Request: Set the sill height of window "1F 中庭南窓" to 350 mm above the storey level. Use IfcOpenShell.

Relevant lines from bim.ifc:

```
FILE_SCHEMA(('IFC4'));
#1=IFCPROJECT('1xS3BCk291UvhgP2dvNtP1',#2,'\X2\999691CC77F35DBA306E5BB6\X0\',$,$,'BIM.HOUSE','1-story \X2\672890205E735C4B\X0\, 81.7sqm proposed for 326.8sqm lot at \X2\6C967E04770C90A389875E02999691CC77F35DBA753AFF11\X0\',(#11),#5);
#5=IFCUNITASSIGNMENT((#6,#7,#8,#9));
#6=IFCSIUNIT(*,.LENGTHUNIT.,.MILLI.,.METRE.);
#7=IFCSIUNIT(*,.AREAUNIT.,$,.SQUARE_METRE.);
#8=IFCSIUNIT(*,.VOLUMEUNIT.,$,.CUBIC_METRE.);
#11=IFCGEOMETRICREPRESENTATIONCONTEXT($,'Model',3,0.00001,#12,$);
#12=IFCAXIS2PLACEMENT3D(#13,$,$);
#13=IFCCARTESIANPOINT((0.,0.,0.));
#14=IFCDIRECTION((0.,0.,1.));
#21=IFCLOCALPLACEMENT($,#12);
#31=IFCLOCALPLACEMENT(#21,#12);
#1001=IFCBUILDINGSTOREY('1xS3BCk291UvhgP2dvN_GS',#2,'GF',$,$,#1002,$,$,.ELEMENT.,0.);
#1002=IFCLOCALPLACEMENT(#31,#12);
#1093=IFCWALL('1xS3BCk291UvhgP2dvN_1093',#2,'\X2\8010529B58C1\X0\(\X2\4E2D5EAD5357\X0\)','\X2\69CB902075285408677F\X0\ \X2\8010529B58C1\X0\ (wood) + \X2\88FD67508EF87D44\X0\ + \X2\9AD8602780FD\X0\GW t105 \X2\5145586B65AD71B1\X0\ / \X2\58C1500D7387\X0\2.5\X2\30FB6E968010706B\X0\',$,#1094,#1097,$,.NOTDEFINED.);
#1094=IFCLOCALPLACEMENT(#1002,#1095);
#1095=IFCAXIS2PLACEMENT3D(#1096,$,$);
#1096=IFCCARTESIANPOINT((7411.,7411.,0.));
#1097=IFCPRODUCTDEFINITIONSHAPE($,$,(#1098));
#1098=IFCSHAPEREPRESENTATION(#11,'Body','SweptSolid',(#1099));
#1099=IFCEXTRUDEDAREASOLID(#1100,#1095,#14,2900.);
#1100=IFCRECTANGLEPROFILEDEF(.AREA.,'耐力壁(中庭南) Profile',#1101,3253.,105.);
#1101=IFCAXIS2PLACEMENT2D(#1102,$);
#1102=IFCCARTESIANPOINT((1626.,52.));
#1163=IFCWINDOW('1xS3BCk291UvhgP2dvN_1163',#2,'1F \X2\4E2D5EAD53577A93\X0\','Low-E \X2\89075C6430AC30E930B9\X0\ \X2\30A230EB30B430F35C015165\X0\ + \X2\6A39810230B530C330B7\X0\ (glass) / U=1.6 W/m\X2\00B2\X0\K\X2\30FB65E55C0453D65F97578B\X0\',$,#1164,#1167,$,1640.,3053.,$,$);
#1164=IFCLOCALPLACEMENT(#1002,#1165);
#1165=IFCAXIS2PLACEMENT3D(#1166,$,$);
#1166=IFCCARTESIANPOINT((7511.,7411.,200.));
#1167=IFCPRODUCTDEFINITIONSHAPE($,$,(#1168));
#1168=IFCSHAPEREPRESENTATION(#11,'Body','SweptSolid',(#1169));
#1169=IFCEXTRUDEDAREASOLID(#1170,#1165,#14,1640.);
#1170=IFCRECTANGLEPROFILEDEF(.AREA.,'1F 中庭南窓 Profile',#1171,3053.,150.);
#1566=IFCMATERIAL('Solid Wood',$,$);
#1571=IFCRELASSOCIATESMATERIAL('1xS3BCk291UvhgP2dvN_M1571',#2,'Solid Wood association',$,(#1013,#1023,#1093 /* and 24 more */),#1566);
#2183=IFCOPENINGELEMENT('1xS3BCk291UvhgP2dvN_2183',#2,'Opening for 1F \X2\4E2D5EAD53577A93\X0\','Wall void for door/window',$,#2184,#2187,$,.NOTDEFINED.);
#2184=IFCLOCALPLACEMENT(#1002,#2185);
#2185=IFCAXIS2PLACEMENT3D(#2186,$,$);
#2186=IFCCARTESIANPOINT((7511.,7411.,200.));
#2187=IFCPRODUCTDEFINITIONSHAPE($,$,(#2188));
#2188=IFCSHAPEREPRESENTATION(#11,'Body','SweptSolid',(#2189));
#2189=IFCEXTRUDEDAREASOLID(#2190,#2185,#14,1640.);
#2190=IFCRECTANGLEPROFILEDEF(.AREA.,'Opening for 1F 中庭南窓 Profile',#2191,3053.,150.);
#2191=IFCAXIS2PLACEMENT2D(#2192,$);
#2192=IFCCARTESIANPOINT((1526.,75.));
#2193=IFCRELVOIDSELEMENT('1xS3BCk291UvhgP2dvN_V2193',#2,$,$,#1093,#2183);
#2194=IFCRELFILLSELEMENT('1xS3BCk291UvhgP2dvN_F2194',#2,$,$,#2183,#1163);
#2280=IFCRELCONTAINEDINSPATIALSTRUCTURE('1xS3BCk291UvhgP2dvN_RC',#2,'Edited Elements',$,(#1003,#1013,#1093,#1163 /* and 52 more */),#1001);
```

```python
import numpy as np
import ifcopenshell
import ifcopenshell.api.geometry
import ifcopenshell.geom
import ifcopenshell.util.element
import ifcopenshell.util.placement
import ifcopenshell.util.shape
import ifcopenshell.util.unit

model = ifcopenshell.open("bim.ifc")
unit_scale = ifcopenshell.util.unit.calculate_unit_scale(model)

window = model.by_guid("1xS3BCk291UvhgP2dvN_1163")
opening = window.FillsVoids[0].RelatingOpeningElement
storey = ifcopenshell.util.element.get_container(window, ifc_class="IfcBuildingStorey")
level = ifcopenshell.util.placement.get_local_placement(storey.ObjectPlacement)[2, 3]

# The opening's origin need not be at the sill, so measure its lowest point.
shape = ifcopenshell.geom.create_shape(ifcopenshell.geom.settings(), opening)
bottom = ifcopenshell.util.shape.get_shape_bottom_elevation(shape, shape.geometry) / unit_scale
dz = level + 0.35 / unit_scale - bottom

shift = np.array([0.0, 0.0, dz])
# The window is not placed relative to its opening, so move both.
for product in (opening, window):
    matrix = ifcopenshell.util.placement.get_local_placement(product.ObjectPlacement)
    matrix[:3, 3] += shift
    ifcopenshell.api.geometry.edit_object_placement(model, product=product, matrix=matrix, is_si=False)

print(f"moved by {dz * unit_scale:+.3f} m")

model.write("bim_updated.ifc")
```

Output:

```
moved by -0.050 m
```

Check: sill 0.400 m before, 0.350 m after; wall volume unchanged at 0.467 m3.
